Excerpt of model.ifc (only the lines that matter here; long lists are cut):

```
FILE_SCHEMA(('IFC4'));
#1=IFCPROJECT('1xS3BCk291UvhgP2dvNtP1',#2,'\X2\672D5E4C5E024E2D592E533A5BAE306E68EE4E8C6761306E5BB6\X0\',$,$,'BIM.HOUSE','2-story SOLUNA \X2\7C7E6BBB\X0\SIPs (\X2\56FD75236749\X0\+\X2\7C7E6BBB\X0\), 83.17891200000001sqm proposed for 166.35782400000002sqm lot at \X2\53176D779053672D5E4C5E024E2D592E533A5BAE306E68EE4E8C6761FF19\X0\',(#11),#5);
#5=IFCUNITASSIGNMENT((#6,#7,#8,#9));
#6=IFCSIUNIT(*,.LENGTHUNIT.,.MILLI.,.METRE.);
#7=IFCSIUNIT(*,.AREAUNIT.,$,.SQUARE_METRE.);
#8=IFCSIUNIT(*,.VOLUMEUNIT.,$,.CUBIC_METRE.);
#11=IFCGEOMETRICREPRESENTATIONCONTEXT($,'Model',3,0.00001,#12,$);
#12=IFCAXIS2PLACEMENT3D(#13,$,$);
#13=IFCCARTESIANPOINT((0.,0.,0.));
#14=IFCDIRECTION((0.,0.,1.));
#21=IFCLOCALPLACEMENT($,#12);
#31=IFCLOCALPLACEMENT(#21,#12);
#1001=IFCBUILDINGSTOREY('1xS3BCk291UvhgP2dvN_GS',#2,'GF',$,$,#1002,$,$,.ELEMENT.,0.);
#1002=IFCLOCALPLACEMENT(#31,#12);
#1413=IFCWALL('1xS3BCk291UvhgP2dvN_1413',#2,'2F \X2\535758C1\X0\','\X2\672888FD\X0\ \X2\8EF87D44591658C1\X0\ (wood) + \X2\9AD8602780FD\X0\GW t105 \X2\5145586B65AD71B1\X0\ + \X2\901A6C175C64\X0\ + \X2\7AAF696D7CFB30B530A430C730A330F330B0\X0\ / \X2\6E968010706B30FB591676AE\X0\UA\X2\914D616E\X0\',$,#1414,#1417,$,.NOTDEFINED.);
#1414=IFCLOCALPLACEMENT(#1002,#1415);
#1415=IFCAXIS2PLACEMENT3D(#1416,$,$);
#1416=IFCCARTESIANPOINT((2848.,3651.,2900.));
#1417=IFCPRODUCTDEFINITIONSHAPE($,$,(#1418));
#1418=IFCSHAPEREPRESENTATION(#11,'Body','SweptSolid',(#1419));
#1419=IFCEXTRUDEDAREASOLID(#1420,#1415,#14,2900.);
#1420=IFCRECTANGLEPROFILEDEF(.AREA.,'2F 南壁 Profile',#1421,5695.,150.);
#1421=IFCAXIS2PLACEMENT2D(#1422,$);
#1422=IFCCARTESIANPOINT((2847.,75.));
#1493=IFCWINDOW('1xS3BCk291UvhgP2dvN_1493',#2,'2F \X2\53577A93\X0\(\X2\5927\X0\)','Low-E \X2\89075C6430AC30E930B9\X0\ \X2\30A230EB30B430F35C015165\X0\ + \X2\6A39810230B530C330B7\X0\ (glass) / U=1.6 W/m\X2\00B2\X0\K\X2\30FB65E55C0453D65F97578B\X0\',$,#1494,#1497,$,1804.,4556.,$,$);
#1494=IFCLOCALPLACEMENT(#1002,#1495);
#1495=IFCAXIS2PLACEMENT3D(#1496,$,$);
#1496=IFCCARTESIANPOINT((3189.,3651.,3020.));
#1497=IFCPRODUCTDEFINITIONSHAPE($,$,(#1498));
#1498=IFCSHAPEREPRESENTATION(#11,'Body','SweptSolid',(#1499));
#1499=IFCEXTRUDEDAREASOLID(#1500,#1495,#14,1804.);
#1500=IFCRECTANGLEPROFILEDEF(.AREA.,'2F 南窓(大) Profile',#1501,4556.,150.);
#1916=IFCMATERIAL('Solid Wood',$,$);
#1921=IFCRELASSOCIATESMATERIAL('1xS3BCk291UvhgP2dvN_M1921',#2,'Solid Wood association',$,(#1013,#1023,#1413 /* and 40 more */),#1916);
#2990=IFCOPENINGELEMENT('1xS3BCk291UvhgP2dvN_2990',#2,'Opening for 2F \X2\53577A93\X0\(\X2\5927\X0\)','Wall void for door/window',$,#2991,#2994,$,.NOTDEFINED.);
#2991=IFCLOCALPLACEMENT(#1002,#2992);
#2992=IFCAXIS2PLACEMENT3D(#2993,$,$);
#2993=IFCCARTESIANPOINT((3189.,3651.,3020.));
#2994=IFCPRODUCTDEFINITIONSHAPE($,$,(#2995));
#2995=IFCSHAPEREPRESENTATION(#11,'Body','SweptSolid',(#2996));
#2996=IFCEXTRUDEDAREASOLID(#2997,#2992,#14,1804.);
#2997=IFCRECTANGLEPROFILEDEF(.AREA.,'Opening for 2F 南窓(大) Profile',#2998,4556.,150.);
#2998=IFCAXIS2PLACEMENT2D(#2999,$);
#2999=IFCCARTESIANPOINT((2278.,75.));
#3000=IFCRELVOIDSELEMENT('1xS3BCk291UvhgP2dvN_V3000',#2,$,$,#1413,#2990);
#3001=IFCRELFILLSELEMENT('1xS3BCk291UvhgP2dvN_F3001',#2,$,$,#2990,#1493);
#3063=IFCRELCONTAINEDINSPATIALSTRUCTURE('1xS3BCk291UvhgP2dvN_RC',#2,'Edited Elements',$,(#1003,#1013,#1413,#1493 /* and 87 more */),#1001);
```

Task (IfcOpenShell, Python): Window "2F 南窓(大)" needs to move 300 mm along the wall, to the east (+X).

```python
import ifcopenshell
import ifcopenshell.api.geometry
import ifcopenshell.util.placement

model = ifcopenshell.open("model.ifc")

window = model.by_id(1493)
opening = window.FillsVoids[0].RelatingOpeningElement
wall = opening.VoidsElements[0].RelatingBuildingElement

wall_matrix = ifcopenshell.util.placement.get_local_placement(wall.ObjectPlacement)
shift = wall_matrix[:3, 0] * 300.0
before = ifcopenshell.util.placement.get_local_placement(window.ObjectPlacement)[:3, 3].copy()

# The window is not placed relative to its opening, so move both.
for product in (opening, window):
    matrix = ifcopenshell.util.placement.get_local_placement(product.ObjectPlacement)
    matrix[:3, 3] += shift
    ifcopenshell.api.geometry.edit_object_placement(model, product=product, matrix=matrix, is_si=False)

after = ifcopenshell.util.placement.get_local_placement(window.ObjectPlacement)[:3, 3]
print("window moved by", (after - before).round(3) + 0.0)

model.write("model_rev.ifc")
```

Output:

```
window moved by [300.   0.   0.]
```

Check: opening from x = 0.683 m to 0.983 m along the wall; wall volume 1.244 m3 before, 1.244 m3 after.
